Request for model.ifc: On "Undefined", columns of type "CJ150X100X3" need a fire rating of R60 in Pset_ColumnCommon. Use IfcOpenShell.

First a look at what the model holds.

```python
import ifcopenshell
import ifcopenshell.util.element

model = ifcopenshell.open("model.ifc")
print(model.schema)
storey = next(s for s in model.by_type("IfcBuildingStorey") if s.Name == "Undefined")
columns = [e for e in ifcopenshell.util.element.get_decomposition(storey) if e.is_a("IfcColumn")]
seen = {}
for e in columns:
    element_type = ifcopenshell.util.element.get_type(e)
    key = (element_type.Name if element_type != e and element_type else None, ifcopenshell.util.element.get_pset(e, "Pset_ColumnCommon", "FireRating"))
    seen[key] = seen.get(key, 0) + 1
for (name, value), count in sorted(seen.items(), key=str):
    print(count, "x", name, "|", value)
```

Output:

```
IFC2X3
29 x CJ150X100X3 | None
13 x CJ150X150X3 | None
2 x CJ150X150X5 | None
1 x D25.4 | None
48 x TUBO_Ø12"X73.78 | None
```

```python
import ifcopenshell
import ifcopenshell.api.pset
import ifcopenshell.util.element

model = ifcopenshell.open("model.ifc")

storey = next(s for s in model.by_type("IfcBuildingStorey") if s.Name == "Undefined")
columns = [e for e in ifcopenshell.util.element.get_decomposition(storey) if e.is_a("IfcColumn")]

count = 0
for e in columns:
    element_type = ifcopenshell.util.element.get_type(e)
    if element_type in (None, e) or element_type.Name != "CJ150X100X3":
        continue
    found = ifcopenshell.util.element.get_pset(e, "Pset_ColumnCommon", should_inherit=False)
    if found:
        pset = model.by_id(found["id"])
        if len(ifcopenshell.util.element.get_elements_by_pset(pset)) > 1:
            pset = ifcopenshell.api.pset.unshare_pset(model, products=[e], pset=pset)[0]
    else:
        pset = ifcopenshell.api.pset.add_pset(model, product=e, name="Pset_ColumnCommon")
    ifcopenshell.api.pset.edit_pset(model, pset=pset, properties={"FireRating": "R60"})
    count += 1

print(count, "columns updated")

model.write("model_rev.ifc")
```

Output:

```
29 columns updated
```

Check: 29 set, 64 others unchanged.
